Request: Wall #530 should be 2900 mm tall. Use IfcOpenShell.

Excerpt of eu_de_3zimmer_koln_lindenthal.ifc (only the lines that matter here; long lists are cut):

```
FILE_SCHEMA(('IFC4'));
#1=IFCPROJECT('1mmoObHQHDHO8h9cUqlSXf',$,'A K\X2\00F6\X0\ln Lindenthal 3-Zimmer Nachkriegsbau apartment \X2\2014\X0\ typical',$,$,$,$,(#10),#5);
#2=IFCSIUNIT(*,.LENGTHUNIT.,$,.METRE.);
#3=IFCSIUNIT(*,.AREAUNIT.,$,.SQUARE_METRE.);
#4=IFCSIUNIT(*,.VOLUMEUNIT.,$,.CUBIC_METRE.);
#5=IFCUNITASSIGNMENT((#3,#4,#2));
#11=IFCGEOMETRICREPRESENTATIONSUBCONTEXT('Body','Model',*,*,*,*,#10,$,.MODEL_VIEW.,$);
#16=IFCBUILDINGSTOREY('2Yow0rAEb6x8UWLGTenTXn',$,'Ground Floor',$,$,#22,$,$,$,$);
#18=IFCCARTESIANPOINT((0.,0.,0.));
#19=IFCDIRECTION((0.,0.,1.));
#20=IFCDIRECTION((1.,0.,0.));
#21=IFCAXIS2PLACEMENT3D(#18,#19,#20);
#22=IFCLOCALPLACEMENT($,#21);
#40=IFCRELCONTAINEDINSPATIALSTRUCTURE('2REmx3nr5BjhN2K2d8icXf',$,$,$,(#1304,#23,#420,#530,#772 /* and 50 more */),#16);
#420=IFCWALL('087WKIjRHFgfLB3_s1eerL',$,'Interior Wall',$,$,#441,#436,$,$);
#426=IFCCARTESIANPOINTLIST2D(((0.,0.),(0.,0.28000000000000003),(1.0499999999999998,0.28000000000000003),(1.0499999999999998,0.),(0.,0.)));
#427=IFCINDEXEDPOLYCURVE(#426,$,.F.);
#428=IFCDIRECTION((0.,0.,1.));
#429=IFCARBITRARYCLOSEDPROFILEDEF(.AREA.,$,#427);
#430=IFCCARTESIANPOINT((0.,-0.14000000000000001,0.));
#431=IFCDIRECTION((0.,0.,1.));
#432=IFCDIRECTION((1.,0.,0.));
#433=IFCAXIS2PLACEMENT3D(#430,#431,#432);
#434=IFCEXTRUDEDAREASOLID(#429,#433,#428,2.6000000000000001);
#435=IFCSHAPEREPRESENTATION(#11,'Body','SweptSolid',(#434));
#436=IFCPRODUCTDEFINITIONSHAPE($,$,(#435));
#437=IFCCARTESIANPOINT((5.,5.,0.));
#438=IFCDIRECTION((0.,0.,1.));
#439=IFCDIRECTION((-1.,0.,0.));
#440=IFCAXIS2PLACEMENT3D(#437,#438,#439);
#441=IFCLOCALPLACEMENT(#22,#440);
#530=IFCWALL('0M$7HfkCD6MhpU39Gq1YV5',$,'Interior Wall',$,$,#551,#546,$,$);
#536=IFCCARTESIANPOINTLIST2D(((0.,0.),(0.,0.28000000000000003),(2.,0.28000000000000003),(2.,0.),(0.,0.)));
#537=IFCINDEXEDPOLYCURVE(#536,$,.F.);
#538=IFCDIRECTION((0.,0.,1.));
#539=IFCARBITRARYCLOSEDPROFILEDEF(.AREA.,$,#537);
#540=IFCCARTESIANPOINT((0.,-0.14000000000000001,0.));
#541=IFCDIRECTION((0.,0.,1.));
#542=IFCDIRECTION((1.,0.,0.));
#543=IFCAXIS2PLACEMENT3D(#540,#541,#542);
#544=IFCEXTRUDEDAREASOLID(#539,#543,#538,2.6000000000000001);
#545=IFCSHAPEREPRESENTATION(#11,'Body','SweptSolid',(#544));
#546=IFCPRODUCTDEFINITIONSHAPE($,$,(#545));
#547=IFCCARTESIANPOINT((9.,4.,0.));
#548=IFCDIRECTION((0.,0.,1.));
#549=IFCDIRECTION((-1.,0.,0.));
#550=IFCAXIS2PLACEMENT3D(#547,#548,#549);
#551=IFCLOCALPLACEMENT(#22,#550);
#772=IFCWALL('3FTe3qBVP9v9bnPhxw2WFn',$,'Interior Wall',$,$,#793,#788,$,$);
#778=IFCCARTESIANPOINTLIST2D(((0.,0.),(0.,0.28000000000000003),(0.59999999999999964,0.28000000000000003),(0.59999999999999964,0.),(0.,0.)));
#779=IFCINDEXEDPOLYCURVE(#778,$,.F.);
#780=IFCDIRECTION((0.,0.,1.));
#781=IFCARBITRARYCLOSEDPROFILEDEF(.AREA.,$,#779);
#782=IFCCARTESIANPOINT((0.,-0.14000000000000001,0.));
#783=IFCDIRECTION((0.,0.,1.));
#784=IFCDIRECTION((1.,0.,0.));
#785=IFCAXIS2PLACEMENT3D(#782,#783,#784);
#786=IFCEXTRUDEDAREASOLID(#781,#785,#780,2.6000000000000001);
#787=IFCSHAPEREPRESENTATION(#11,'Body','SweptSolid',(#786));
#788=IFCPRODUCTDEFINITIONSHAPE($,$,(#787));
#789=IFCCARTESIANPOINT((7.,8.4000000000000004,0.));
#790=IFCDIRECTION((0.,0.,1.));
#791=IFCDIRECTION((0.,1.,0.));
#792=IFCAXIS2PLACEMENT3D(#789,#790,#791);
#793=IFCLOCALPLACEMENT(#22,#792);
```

```python
import ifcopenshell
import ifcopenshell.geom
import ifcopenshell.util.representation
import ifcopenshell.util.shape

model = ifcopenshell.open("eu_de_3zimmer_koln_lindenthal.ifc")
settings = ifcopenshell.geom.settings()


def volume(element):
    """Net volume in cubic metres, openings subtracted."""
    shape = ifcopenshell.geom.create_shape(settings, element)
    return ifcopenshell.util.shape.get_volume(shape.geometry)


wall = model.by_guid("0M$7HfkCD6MhpU39Gq1YV5")
before = volume(wall)

body = ifcopenshell.util.representation.get_representation(wall, "Model", "Body")
solid = body.Items[0]
old_height = solid.Depth
solid.Depth = 2.9
after = volume(wall)

print(f"height {old_height:g} -> {solid.Depth:g}, volume {before:.3f} -> {after:.3f} m3")

model.write("eu_de_3zimmer_koln_lindenthal_edited.ifc")
```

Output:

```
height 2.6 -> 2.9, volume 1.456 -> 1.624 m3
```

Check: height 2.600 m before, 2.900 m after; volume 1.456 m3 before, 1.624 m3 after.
